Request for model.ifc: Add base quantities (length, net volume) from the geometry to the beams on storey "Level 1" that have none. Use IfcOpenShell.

First a look at what the model holds.

```python
import ifcopenshell
import ifcopenshell.util.element
import ifcopenshell.util.unit

model = ifcopenshell.open("model.ifc")
print(model.schema)
for unit_type in ("LENGTHUNIT", "AREAUNIT", "VOLUMEUNIT"):
    print(unit_type, ifcopenshell.util.unit.calculate_unit_scale(model, unit_type))
storey = next(s for s in model.by_type("IfcBuildingStorey") if s.Name == "Level 1")
beams = [e for e in ifcopenshell.util.element.get_decomposition(storey) if e.is_a("IfcBeam")]
for e in sorted(beams, key=lambda e: e.id()):
    print(e.id(), e.is_a(), e.Name, list(ifcopenshell.util.element.get_psets(e, qtos_only=True)), sep=" | ")
```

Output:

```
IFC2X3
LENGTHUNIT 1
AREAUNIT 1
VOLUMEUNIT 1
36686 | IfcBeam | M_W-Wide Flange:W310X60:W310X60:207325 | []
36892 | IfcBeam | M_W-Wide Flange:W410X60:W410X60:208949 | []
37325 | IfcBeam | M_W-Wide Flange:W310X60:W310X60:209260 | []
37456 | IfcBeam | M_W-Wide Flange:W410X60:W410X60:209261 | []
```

```python
import ifcopenshell
import ifcopenshell.api.pset
import ifcopenshell.geom
import ifcopenshell.util.element
import ifcopenshell.util.shape
import ifcopenshell.util.unit

model = ifcopenshell.open("model.ifc")
unit_scale = ifcopenshell.util.unit.calculate_unit_scale(model)
volume_scale = ifcopenshell.util.unit.calculate_unit_scale(model, "VOLUMEUNIT")
settings = ifcopenshell.geom.settings()

storey = next(s for s in model.by_type("IfcBuildingStorey") if s.Name == "Level 1")
beams = [e for e in ifcopenshell.util.element.get_decomposition(storey) if e.is_a("IfcBeam")]

for e in sorted(beams, key=lambda e: e.id()):
    if ifcopenshell.util.element.get_psets(e, qtos_only=True, should_inherit=False):
        continue
    # Geometry comes back in metres, in the element's own axes.
    shape = ifcopenshell.geom.create_shape(settings, e)
    values = {
        "Length": ifcopenshell.util.shape.get_max_xyz(shape.geometry) / unit_scale,
        "NetVolume": ifcopenshell.util.shape.get_volume(shape.geometry) / volume_scale,
    }
    qto = ifcopenshell.api.pset.add_qto(model, product=e, name="BaseQuantities")
    ifcopenshell.api.pset.edit_qto(model, qto=qto, properties=values)
    print(e.id(), {k: round(v, 3) for k, v in values.items()})

model.write("model-out.ifc")
```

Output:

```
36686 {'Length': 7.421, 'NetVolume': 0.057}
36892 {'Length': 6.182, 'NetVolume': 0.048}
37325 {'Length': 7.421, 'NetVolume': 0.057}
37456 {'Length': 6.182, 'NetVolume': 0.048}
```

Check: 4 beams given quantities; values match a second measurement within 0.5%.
